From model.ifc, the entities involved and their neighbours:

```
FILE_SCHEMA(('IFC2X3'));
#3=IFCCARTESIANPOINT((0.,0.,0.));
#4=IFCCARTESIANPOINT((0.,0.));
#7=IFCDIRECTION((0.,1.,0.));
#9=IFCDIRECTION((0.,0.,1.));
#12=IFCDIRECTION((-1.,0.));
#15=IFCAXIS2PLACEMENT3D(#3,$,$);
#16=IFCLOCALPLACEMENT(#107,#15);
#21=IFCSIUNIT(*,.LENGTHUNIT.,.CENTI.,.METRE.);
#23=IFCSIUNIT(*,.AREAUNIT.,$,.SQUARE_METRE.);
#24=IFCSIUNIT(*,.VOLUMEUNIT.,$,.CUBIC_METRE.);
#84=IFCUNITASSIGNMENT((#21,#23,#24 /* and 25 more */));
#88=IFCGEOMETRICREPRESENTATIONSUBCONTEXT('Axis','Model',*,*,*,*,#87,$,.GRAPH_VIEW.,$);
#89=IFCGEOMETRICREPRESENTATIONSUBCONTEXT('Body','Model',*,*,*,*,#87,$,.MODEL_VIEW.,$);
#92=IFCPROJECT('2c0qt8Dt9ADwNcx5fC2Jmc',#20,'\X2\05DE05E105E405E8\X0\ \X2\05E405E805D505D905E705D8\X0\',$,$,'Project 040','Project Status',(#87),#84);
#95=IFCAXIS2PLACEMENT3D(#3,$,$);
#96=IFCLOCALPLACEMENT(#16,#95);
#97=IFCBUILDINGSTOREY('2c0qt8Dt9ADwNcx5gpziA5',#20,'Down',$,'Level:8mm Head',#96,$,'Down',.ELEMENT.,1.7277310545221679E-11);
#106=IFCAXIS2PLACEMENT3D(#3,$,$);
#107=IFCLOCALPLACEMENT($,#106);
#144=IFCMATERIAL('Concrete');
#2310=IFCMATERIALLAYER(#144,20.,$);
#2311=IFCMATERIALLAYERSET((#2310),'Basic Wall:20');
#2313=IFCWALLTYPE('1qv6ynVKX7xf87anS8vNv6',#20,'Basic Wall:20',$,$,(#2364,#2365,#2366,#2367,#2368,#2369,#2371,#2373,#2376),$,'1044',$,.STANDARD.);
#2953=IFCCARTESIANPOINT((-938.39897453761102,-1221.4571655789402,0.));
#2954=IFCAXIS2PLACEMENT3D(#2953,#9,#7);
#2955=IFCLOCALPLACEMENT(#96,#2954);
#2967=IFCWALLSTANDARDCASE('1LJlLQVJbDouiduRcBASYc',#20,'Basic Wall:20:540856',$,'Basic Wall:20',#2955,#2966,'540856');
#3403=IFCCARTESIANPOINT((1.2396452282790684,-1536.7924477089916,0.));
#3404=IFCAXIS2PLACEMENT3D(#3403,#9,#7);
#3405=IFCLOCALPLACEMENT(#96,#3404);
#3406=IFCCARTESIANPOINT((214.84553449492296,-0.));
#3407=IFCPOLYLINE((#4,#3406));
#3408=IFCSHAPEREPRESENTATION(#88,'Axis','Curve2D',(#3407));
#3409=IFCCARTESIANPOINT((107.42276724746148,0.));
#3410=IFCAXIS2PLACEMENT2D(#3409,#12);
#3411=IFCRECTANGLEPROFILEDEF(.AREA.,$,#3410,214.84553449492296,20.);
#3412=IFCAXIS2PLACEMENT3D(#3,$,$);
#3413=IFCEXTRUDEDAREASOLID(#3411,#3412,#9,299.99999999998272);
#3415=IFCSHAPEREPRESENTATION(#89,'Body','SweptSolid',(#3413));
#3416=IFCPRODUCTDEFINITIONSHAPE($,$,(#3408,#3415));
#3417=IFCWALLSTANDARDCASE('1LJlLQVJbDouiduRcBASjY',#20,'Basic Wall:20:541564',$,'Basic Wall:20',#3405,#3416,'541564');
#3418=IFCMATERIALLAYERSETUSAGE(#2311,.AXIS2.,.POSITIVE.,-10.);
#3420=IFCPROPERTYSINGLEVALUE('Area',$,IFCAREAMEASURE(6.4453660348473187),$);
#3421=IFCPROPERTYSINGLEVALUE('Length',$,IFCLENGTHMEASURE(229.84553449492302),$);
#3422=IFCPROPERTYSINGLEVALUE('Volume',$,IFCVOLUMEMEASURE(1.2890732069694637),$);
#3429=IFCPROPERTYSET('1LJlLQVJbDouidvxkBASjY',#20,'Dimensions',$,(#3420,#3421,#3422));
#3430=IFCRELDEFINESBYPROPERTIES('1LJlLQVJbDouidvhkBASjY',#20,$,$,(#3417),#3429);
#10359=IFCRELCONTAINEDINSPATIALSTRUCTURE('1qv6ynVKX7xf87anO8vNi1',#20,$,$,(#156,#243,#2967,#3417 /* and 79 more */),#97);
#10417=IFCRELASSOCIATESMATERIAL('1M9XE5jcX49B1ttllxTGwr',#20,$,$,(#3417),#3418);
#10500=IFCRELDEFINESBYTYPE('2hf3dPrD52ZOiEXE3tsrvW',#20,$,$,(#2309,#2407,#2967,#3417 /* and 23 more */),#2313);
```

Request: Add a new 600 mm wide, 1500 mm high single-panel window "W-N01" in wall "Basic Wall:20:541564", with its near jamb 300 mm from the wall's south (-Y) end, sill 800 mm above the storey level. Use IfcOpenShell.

```python
import numpy as np
import ifcopenshell
import ifcopenshell.api.feature
import ifcopenshell.api.geometry
import ifcopenshell.api.pset
import ifcopenshell.api.root
import ifcopenshell.api.spatial
import ifcopenshell.api.type
import ifcopenshell.geom
import ifcopenshell.util.element
import ifcopenshell.util.placement
import ifcopenshell.util.representation
import ifcopenshell.util.shape
import ifcopenshell.util.unit

model = ifcopenshell.open("model.ifc")
unit_scale = ifcopenshell.util.unit.calculate_unit_scale(model)
area_scale = ifcopenshell.util.unit.calculate_unit_scale(model, "AREAUNIT")
volume_scale = ifcopenshell.util.unit.calculate_unit_scale(model, "VOLUMEUNIT")
settings = ifcopenshell.geom.settings()


def volume(element):
    """Net volume in cubic metres, openings subtracted."""
    shape = ifcopenshell.geom.create_shape(settings, element)
    return ifcopenshell.util.shape.get_volume(shape.geometry)


wall = model.by_guid("1LJlLQVJbDouiduRcBASjY")
storey = ifcopenshell.util.element.get_container(wall, ifc_class="IfcBuildingStorey")
context = ifcopenshell.util.representation.get_context(model, "Model", "Body", "MODEL_VIEW")
before = volume(wall)

width, height, from_end, sill = 0.6, 1.5, 0.3, 0.8  # metres

# The wall runs along its own X axis, and the end named is its -X end.
wall_shape = ifcopenshell.geom.create_shape(settings, wall)
x, y, z = ifcopenshell.util.shape.get_vertices(wall_shape.geometry).T
start = x.min() + from_end
face, thickness = float(y.min()), float(y.max() - y.min())
wall_matrix = ifcopenshell.util.placement.get_local_placement(wall.ObjectPlacement)
level = ifcopenshell.util.placement.get_local_placement(storey.ObjectPlacement)[2, 3]


def in_wall(x, y):
    """Placement at x, y metres in the wall's axes, at sill height."""
    matrix = wall_matrix.copy()
    matrix[:, 3] = wall_matrix @ np.array([x / unit_scale, y / unit_scale, 0.0, 1.0])
    matrix[2, 3] = level + sill / unit_scale
    return matrix


# Opening: a box that overshoots both wall faces by 50 mm.
opening = ifcopenshell.api.root.create_entity(model, ifc_class="IfcOpeningElement")
box = ifcopenshell.api.geometry.add_wall_representation(
    model, context=context, length=width, height=height, thickness=thickness + 0.1
)
ifcopenshell.api.geometry.assign_representation(model, product=opening, representation=box)
ifcopenshell.api.geometry.edit_object_placement(model, product=opening, matrix=in_wall(start, face - 0.05), is_si=False)
ifcopenshell.api.feature.add_feature(model, feature=opening, element=wall)

window = ifcopenshell.api.root.create_entity(model, ifc_class="IfcWindow", name="W-N01")
window.OverallWidth, window.OverallHeight = width / unit_scale, height / unit_scale
body = ifcopenshell.api.geometry.add_window_representation(
    model,
    context=context,
    overall_width=window.OverallWidth,
    overall_height=window.OverallHeight,
    partition_type="SINGLE_PANEL",
)
ifcopenshell.api.geometry.assign_representation(model, product=window, representation=body)
ifcopenshell.api.spatial.assign_container(model, products=[window], relating_structure=storey)
fills = ifcopenshell.api.feature.add_filling(model, opening=opening, element=window)
fills.OwnerHistory = window.OwnerHistory  # required in IFC2X3

# IFC2X3 keeps the operation on the window style.
style = ifcopenshell.api.root.create_entity(model, ifc_class="IfcWindowStyle", name="W-N01")
style.OperationType, style.ConstructionType = "SINGLE_PANEL", "NOTDEFINED"
style.ParameterTakesPrecedence = style.Sizeable = False
ifcopenshell.api.type.assign_type(model, related_objects=[window], relating_type=style)

# Centre the window in the wall's thickness.
ifcopenshell.api.geometry.edit_object_placement(model, product=window, matrix=in_wall(start, face), is_si=False)
window_shape = ifcopenshell.geom.create_shape(settings, window)
depth = ifcopenshell.util.shape.get_vertices(window_shape.geometry)[:, 1]
offset = face + thickness / 2 - (depth.min() + depth.max()) / 2
ifcopenshell.api.geometry.edit_object_placement(model, product=window, matrix=in_wall(start, offset), is_si=False)

after = volume(wall)

# Update the wall's stored quantities.
pset = model.by_id(ifcopenshell.util.element.get_pset(wall, "Dimensions", should_inherit=False)["id"])
ifcopenshell.api.pset.edit_pset(model, pset=pset, properties={
    "Area": model.create_entity("IfcAreaMeasure", after / thickness / area_scale),
    "Volume": model.create_entity("IfcVolumeMeasure", after / volume_scale),
})

print(f"wall volume {before:.3f} -> {after:.3f} m3")

model.write("model_updated.ifc")
```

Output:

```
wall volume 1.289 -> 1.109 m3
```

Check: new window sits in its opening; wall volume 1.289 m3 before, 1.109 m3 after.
